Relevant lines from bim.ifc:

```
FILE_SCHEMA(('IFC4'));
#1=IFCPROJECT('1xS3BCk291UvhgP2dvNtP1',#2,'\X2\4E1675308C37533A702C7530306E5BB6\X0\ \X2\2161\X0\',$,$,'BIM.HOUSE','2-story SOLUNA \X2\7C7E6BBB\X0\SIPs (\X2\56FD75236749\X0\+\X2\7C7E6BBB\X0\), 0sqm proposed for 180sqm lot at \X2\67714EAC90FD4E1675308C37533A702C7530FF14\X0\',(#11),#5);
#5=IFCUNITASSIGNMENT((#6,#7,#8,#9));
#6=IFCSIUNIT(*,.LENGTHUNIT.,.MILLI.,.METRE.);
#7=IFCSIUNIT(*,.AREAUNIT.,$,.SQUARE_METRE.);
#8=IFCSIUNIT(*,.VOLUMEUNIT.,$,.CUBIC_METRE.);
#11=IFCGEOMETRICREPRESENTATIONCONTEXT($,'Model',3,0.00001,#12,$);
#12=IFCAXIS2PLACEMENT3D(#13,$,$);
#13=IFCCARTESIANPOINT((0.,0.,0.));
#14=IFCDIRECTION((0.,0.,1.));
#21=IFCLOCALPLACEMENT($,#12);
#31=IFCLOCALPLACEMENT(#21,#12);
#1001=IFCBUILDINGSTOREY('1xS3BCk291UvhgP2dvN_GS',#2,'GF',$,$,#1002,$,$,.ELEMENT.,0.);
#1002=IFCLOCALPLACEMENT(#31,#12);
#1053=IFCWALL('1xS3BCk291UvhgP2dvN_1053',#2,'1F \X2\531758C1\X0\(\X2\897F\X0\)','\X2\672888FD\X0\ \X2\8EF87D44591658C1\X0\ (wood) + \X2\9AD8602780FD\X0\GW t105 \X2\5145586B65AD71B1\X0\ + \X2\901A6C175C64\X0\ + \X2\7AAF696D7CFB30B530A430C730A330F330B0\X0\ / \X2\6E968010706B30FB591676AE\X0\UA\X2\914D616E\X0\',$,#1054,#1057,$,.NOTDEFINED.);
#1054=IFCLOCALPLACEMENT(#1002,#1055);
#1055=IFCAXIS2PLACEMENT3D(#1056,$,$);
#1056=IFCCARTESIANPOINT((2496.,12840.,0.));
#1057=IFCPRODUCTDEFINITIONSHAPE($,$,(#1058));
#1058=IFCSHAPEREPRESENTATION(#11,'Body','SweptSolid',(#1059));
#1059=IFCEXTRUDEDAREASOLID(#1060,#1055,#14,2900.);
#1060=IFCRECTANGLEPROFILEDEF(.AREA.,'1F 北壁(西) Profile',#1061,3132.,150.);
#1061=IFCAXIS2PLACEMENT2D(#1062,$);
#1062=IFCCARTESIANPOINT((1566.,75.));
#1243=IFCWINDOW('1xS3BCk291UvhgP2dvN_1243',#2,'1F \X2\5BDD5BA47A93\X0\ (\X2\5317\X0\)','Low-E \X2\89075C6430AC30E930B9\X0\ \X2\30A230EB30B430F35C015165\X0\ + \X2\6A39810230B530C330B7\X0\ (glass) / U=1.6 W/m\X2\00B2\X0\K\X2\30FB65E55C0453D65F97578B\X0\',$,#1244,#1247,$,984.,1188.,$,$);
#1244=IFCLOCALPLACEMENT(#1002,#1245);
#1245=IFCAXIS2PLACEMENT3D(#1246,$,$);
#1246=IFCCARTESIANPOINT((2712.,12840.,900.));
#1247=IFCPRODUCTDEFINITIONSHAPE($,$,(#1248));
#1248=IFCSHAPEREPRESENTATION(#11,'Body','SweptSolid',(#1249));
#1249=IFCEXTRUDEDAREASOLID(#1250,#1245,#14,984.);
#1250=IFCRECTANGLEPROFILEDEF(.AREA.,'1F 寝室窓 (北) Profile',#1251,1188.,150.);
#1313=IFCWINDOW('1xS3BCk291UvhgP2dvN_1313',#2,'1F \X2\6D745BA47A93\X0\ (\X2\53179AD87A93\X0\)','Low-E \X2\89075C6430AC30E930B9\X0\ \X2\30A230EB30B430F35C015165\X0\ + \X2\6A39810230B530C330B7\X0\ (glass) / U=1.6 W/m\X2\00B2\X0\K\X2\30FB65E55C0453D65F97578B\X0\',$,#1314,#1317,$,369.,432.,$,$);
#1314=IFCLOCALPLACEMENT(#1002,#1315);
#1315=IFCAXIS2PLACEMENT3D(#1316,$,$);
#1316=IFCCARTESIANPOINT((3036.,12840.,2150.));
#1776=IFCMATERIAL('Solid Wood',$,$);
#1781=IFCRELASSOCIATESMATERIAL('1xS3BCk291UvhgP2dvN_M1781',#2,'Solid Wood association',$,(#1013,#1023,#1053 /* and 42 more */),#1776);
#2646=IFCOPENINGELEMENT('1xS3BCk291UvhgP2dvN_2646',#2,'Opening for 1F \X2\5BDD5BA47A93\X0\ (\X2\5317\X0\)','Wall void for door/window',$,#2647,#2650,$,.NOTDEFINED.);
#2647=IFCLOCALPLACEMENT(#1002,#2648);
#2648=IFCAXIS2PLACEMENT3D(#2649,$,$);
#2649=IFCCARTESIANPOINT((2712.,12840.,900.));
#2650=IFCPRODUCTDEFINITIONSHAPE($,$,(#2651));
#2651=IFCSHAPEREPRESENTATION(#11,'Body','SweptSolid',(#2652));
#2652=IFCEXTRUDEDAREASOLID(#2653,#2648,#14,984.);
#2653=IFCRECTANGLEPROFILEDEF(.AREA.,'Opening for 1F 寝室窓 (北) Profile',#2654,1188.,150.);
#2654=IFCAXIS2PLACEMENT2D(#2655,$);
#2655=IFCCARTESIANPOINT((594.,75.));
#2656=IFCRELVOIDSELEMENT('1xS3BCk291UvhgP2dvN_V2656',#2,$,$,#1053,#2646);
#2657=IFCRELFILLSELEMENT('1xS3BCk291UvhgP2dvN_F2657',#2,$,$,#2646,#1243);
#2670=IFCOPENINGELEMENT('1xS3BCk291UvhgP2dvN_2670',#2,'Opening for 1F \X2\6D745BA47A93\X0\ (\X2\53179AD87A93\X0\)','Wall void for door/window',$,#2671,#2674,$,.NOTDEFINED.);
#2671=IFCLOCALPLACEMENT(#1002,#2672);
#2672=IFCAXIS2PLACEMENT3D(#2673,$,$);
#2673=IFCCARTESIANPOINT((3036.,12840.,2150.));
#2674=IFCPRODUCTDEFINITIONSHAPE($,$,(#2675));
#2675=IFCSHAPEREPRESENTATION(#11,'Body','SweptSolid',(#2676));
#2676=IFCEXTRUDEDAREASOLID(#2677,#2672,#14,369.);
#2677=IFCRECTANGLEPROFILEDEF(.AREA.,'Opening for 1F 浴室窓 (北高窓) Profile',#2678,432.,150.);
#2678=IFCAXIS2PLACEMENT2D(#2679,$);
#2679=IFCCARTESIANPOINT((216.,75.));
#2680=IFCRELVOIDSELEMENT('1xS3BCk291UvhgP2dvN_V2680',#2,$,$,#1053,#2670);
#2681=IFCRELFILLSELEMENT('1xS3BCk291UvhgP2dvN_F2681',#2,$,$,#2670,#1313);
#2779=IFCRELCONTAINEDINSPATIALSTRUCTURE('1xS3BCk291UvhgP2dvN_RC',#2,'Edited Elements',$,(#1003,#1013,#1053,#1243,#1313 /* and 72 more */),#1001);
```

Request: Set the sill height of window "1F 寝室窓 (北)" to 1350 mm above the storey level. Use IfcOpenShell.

```python
import numpy as np
import ifcopenshell
import ifcopenshell.api.geometry
import ifcopenshell.geom
import ifcopenshell.util.element
import ifcopenshell.util.placement
import ifcopenshell.util.shape
import ifcopenshell.util.unit

model = ifcopenshell.open("bim.ifc")
unit_scale = ifcopenshell.util.unit.calculate_unit_scale(model)

window = model.by_guid("1xS3BCk291UvhgP2dvN_1243")
opening = window.FillsVoids[0].RelatingOpeningElement
storey = ifcopenshell.util.element.get_container(window, ifc_class="IfcBuildingStorey")
level = ifcopenshell.util.placement.get_local_placement(storey.ObjectPlacement)[2, 3]

# The opening's origin need not be at the sill, so measure its lowest point.
shape = ifcopenshell.geom.create_shape(ifcopenshell.geom.settings(), opening)
bottom = ifcopenshell.util.shape.get_shape_bottom_elevation(shape, shape.geometry) / unit_scale
dz = level + 1.35 / unit_scale - bottom

shift = np.array([0.0, 0.0, dz])
# The window is not placed relative to its opening, so move both.
for product in (opening, window):
    matrix = ifcopenshell.util.placement.get_local_placement(product.ObjectPlacement)
    matrix[:3, 3] += shift
    ifcopenshell.api.geometry.edit_object_placement(model, product=product, matrix=matrix, is_si=False)

print(f"moved by {dz * unit_scale:+.3f} m")

model.write("bim_edited.ifc")
```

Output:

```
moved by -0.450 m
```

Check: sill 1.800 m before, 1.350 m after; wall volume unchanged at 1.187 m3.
